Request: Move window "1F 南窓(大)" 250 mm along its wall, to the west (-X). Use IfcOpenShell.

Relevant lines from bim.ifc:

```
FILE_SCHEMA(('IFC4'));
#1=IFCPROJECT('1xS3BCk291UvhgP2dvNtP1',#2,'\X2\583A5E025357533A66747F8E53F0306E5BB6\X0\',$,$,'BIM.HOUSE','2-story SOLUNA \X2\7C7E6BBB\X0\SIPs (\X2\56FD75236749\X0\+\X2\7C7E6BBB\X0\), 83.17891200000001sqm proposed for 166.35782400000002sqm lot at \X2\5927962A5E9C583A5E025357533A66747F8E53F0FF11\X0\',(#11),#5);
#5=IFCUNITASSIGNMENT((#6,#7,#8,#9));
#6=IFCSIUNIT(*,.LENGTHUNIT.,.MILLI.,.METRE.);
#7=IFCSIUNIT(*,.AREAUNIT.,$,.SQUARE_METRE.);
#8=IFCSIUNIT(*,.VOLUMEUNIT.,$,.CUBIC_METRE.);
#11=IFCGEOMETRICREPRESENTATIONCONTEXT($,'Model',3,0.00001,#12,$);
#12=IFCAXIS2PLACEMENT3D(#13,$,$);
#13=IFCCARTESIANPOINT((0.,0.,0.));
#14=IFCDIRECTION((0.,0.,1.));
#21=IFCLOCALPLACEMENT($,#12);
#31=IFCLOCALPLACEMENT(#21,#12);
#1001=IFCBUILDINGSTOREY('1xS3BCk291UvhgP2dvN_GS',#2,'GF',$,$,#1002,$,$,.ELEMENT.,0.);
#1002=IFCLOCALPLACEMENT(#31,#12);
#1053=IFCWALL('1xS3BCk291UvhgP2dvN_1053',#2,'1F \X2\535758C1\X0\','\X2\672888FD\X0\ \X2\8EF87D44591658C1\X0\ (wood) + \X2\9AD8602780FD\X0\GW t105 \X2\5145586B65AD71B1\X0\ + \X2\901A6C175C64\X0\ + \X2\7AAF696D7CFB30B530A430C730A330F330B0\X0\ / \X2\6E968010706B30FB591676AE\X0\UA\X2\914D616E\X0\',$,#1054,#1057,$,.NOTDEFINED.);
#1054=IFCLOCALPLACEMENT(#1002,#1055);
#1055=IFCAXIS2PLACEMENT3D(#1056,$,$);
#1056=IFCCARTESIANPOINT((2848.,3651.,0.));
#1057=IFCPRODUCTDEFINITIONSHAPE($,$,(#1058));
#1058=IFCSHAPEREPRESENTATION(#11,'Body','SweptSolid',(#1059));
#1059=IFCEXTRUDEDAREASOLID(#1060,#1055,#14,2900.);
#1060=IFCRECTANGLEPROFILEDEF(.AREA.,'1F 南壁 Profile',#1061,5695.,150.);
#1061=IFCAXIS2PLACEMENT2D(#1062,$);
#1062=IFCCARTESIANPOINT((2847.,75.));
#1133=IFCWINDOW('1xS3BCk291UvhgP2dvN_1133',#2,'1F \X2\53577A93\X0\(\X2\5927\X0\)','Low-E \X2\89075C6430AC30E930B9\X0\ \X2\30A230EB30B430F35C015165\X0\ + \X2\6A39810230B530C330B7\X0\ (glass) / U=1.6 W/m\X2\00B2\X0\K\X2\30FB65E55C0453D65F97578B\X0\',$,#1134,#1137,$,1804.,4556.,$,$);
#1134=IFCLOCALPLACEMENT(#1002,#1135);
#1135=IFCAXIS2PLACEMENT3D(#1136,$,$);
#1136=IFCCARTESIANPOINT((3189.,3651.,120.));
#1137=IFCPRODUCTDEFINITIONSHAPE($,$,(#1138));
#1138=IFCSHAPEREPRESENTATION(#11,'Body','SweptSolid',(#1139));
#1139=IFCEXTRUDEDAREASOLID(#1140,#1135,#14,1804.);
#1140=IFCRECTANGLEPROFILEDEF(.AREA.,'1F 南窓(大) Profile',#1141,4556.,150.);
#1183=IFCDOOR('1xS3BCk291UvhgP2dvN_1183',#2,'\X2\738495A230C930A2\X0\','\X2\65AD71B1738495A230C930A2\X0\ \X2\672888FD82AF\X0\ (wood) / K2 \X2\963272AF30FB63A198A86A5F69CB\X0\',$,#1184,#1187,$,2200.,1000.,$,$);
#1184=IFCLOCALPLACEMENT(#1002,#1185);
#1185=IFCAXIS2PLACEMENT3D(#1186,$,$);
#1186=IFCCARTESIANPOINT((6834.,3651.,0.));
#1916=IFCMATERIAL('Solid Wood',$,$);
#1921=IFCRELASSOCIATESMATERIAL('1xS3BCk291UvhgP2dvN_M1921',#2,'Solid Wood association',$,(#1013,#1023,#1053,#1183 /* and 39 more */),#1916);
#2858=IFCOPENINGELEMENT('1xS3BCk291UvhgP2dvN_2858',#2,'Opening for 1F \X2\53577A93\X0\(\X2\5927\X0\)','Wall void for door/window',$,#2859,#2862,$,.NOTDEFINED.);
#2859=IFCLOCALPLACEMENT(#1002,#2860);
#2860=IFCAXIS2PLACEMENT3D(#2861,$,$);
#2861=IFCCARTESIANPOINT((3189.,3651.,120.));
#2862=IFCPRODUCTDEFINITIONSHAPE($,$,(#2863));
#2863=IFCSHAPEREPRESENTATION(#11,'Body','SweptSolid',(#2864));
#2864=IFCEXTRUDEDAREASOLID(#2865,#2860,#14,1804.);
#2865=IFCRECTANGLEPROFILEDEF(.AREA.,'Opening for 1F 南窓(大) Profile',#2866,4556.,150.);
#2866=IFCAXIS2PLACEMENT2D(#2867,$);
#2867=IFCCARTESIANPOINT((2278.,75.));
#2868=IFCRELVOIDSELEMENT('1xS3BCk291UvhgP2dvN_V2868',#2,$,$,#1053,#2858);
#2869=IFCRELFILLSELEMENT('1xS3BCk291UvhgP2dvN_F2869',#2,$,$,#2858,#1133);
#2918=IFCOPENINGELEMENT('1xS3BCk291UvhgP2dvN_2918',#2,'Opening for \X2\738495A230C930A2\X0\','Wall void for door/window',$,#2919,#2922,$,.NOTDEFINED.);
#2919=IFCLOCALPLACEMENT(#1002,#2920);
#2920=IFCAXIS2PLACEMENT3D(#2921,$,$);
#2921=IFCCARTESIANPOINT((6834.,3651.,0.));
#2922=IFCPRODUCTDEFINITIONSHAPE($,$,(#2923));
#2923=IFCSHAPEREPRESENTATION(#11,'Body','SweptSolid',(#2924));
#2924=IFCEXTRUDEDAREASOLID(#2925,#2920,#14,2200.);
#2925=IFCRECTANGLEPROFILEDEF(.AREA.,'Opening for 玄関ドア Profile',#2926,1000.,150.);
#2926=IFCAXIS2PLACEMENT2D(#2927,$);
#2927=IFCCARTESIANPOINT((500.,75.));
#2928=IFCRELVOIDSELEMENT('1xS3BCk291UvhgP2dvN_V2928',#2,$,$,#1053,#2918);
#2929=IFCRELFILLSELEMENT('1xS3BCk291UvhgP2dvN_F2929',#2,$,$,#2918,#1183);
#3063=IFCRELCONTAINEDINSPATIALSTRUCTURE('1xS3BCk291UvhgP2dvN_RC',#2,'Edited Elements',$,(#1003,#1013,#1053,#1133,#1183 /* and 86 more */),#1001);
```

```python
import ifcopenshell
import ifcopenshell.api.geometry
import ifcopenshell.util.placement

model = ifcopenshell.open("bim.ifc")

window = model.by_guid("1xS3BCk291UvhgP2dvN_1133")
opening = window.FillsVoids[0].RelatingOpeningElement
wall = opening.VoidsElements[0].RelatingBuildingElement

wall_matrix = ifcopenshell.util.placement.get_local_placement(wall.ObjectPlacement)
shift = wall_matrix[:3, 0] * -250.0
before = ifcopenshell.util.placement.get_local_placement(window.ObjectPlacement)[:3, 3].copy()

# The window is not placed relative to its opening, so move both.
for product in (opening, window):
    matrix = ifcopenshell.util.placement.get_local_placement(product.ObjectPlacement)
    matrix[:3, 3] += shift
    ifcopenshell.api.geometry.edit_object_placement(model, product=product, matrix=matrix, is_si=False)

after = ifcopenshell.util.placement.get_local_placement(window.ObjectPlacement)[:3, 3]
print("window moved by", (after - before).round(3) + 0.0)

model.write("bim-out.ifc")
```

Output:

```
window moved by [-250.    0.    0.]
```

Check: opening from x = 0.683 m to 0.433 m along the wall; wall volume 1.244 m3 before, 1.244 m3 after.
